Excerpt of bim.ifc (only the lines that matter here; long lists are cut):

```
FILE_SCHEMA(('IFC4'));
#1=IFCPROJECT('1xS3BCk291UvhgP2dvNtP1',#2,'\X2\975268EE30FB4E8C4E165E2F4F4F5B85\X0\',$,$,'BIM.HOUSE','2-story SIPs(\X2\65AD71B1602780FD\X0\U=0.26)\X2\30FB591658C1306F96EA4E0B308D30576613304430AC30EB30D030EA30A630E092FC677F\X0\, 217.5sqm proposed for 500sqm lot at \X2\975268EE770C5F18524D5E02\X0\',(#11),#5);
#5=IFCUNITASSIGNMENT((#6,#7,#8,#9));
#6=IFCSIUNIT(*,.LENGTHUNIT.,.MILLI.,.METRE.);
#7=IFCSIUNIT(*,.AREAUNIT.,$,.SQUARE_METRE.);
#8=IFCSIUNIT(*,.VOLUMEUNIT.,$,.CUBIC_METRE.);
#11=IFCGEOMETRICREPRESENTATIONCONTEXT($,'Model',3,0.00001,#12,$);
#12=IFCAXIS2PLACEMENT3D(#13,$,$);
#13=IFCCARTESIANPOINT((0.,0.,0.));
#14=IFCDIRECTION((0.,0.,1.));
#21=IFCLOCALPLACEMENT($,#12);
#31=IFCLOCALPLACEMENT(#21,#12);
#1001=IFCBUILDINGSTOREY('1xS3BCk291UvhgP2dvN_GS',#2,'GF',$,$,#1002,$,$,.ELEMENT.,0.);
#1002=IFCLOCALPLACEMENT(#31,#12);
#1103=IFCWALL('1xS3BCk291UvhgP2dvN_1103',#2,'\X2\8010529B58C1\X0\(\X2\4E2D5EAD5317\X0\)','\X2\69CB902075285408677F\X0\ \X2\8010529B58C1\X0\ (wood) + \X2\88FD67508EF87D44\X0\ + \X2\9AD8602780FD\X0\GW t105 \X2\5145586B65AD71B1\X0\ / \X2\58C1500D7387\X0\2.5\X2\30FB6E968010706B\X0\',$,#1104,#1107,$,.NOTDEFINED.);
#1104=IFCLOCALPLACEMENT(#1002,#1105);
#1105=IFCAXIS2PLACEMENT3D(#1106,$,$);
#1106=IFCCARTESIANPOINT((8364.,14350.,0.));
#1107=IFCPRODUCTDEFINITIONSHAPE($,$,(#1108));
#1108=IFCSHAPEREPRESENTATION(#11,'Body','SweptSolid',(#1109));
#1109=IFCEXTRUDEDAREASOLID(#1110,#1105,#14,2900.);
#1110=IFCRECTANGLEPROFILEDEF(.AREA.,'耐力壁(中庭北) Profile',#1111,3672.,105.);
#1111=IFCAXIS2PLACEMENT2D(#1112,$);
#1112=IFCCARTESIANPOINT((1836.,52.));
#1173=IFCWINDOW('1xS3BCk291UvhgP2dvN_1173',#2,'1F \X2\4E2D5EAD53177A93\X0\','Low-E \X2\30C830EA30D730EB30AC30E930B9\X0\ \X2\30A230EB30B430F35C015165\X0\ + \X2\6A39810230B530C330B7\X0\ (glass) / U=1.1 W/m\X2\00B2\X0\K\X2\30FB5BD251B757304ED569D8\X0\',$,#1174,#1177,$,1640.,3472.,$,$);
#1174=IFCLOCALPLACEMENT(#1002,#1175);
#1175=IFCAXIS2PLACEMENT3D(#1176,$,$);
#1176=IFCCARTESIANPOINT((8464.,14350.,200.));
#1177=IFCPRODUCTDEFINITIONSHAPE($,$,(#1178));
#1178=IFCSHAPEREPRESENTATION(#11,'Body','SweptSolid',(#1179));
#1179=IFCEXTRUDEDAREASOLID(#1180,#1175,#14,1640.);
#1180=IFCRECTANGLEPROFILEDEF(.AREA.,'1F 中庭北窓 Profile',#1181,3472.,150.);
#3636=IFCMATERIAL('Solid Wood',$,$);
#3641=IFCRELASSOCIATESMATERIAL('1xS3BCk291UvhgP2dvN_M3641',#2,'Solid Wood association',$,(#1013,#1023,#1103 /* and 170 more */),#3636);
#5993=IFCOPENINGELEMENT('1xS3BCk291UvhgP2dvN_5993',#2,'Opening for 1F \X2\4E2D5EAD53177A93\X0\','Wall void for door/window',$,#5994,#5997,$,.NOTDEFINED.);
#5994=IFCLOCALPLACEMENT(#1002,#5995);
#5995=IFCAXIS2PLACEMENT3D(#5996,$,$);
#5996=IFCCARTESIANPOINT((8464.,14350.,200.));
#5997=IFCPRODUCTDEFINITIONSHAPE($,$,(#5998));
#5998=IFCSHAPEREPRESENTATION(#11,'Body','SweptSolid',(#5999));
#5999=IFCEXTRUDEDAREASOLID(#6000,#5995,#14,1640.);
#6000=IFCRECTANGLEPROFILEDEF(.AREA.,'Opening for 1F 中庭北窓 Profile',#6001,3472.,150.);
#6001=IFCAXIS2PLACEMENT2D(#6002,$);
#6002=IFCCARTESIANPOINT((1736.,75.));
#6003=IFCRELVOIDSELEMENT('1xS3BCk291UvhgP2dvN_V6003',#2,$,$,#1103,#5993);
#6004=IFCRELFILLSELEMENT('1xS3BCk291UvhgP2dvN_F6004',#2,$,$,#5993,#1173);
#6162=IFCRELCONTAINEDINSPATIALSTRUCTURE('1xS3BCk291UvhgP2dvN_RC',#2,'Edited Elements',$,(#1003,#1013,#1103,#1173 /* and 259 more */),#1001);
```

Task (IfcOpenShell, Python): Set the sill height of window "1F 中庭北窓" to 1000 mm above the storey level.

```python
import numpy as np
import ifcopenshell
import ifcopenshell.api.geometry
import ifcopenshell.geom
import ifcopenshell.util.element
import ifcopenshell.util.placement
import ifcopenshell.util.shape
import ifcopenshell.util.unit

model = ifcopenshell.open("bim.ifc")
unit_scale = ifcopenshell.util.unit.calculate_unit_scale(model)

window = model.by_guid("1xS3BCk291UvhgP2dvN_1173")
opening = window.FillsVoids[0].RelatingOpeningElement
storey = ifcopenshell.util.element.get_container(window, ifc_class="IfcBuildingStorey")
level = ifcopenshell.util.placement.get_local_placement(storey.ObjectPlacement)[2, 3]

# The opening's origin need not be at the sill, so measure its lowest point.
shape = ifcopenshell.geom.create_shape(ifcopenshell.geom.settings(), opening)
bottom = ifcopenshell.util.shape.get_shape_bottom_elevation(shape, shape.geometry) / unit_scale
dz = level + 1000.0 - bottom

shift = np.array([0.0, 0.0, dz])
# The window is not placed relative to its opening, so move both.
for product in (opening, window):
    matrix = ifcopenshell.util.placement.get_local_placement(product.ObjectPlacement)
    matrix[:3, 3] += shift
    ifcopenshell.api.geometry.edit_object_placement(model, product=product, matrix=matrix, is_si=False)

print(f"moved by {dz * unit_scale:+.3f} m")

model.write("bim_rev.ifc")
```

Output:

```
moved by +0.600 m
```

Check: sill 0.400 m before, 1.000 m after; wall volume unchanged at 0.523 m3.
